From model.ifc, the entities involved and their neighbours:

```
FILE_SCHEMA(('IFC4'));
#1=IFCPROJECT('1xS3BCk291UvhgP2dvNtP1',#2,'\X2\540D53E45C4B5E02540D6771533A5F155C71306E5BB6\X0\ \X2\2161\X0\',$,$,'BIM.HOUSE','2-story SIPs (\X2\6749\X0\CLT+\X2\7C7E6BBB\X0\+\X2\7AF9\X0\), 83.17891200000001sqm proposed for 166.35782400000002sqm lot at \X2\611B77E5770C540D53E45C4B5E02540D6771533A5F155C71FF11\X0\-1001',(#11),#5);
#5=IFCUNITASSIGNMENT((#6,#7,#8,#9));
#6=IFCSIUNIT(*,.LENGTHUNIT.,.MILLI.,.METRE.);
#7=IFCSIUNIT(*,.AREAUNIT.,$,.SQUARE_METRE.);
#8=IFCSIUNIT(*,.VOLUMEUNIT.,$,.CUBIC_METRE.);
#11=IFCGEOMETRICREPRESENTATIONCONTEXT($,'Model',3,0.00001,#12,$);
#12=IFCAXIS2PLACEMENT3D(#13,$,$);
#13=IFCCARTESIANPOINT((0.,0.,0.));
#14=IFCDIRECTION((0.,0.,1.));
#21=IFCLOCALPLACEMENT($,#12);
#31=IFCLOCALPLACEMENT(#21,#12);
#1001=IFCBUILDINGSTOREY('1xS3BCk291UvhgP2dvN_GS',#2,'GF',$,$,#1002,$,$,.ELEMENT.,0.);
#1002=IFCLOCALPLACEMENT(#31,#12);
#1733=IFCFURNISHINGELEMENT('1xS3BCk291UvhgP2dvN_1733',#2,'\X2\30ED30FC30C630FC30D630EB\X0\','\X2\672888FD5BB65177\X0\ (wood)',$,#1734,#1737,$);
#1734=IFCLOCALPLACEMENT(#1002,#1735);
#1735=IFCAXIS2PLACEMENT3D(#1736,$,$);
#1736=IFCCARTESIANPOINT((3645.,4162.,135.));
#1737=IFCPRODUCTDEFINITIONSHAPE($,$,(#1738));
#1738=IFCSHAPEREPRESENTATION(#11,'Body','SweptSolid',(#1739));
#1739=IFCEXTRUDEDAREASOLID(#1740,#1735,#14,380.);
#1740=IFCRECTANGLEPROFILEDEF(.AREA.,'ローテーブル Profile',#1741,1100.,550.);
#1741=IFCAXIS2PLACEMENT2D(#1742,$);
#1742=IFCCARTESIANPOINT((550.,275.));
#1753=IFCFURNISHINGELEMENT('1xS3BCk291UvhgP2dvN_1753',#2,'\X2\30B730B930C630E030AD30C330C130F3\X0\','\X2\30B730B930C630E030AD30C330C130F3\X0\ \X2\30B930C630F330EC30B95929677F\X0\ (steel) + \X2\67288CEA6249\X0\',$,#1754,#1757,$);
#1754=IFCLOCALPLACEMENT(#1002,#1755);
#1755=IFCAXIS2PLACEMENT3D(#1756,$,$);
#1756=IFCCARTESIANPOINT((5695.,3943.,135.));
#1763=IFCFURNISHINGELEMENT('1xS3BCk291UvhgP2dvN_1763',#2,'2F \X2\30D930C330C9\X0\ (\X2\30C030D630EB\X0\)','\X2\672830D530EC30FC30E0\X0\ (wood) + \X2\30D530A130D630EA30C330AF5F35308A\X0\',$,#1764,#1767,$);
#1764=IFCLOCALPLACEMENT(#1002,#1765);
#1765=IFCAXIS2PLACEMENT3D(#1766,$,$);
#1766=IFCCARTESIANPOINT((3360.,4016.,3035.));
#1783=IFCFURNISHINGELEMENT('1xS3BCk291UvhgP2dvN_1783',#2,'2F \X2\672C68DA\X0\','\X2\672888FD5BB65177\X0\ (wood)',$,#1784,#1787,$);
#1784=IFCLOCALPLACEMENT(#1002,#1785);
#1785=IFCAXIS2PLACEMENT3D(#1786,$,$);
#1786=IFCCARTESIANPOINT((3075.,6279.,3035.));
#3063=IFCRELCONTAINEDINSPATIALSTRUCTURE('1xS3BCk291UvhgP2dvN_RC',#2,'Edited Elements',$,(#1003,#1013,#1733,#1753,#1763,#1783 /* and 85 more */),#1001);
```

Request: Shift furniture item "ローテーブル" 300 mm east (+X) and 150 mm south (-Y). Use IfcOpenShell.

```python
import ifcopenshell
import ifcopenshell.api.geometry
import ifcopenshell.util.placement

model = ifcopenshell.open("model.ifc")

item = model.by_guid("1xS3BCk291UvhgP2dvN_1733")
matrix = ifcopenshell.util.placement.get_local_placement(item.ObjectPlacement)
matrix[0, 3] += 300.0
matrix[1, 3] -= 150.0
ifcopenshell.api.geometry.edit_object_placement(model, product=item, matrix=matrix, is_si=False)

print(ifcopenshell.util.placement.get_local_placement(item.ObjectPlacement).round(3) + 0.0)

model.write("model_v2.ifc")
```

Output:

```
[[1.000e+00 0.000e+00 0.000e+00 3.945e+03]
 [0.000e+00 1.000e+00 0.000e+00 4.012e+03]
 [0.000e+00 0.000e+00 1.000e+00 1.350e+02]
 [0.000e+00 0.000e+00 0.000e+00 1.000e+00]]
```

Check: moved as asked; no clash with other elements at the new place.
